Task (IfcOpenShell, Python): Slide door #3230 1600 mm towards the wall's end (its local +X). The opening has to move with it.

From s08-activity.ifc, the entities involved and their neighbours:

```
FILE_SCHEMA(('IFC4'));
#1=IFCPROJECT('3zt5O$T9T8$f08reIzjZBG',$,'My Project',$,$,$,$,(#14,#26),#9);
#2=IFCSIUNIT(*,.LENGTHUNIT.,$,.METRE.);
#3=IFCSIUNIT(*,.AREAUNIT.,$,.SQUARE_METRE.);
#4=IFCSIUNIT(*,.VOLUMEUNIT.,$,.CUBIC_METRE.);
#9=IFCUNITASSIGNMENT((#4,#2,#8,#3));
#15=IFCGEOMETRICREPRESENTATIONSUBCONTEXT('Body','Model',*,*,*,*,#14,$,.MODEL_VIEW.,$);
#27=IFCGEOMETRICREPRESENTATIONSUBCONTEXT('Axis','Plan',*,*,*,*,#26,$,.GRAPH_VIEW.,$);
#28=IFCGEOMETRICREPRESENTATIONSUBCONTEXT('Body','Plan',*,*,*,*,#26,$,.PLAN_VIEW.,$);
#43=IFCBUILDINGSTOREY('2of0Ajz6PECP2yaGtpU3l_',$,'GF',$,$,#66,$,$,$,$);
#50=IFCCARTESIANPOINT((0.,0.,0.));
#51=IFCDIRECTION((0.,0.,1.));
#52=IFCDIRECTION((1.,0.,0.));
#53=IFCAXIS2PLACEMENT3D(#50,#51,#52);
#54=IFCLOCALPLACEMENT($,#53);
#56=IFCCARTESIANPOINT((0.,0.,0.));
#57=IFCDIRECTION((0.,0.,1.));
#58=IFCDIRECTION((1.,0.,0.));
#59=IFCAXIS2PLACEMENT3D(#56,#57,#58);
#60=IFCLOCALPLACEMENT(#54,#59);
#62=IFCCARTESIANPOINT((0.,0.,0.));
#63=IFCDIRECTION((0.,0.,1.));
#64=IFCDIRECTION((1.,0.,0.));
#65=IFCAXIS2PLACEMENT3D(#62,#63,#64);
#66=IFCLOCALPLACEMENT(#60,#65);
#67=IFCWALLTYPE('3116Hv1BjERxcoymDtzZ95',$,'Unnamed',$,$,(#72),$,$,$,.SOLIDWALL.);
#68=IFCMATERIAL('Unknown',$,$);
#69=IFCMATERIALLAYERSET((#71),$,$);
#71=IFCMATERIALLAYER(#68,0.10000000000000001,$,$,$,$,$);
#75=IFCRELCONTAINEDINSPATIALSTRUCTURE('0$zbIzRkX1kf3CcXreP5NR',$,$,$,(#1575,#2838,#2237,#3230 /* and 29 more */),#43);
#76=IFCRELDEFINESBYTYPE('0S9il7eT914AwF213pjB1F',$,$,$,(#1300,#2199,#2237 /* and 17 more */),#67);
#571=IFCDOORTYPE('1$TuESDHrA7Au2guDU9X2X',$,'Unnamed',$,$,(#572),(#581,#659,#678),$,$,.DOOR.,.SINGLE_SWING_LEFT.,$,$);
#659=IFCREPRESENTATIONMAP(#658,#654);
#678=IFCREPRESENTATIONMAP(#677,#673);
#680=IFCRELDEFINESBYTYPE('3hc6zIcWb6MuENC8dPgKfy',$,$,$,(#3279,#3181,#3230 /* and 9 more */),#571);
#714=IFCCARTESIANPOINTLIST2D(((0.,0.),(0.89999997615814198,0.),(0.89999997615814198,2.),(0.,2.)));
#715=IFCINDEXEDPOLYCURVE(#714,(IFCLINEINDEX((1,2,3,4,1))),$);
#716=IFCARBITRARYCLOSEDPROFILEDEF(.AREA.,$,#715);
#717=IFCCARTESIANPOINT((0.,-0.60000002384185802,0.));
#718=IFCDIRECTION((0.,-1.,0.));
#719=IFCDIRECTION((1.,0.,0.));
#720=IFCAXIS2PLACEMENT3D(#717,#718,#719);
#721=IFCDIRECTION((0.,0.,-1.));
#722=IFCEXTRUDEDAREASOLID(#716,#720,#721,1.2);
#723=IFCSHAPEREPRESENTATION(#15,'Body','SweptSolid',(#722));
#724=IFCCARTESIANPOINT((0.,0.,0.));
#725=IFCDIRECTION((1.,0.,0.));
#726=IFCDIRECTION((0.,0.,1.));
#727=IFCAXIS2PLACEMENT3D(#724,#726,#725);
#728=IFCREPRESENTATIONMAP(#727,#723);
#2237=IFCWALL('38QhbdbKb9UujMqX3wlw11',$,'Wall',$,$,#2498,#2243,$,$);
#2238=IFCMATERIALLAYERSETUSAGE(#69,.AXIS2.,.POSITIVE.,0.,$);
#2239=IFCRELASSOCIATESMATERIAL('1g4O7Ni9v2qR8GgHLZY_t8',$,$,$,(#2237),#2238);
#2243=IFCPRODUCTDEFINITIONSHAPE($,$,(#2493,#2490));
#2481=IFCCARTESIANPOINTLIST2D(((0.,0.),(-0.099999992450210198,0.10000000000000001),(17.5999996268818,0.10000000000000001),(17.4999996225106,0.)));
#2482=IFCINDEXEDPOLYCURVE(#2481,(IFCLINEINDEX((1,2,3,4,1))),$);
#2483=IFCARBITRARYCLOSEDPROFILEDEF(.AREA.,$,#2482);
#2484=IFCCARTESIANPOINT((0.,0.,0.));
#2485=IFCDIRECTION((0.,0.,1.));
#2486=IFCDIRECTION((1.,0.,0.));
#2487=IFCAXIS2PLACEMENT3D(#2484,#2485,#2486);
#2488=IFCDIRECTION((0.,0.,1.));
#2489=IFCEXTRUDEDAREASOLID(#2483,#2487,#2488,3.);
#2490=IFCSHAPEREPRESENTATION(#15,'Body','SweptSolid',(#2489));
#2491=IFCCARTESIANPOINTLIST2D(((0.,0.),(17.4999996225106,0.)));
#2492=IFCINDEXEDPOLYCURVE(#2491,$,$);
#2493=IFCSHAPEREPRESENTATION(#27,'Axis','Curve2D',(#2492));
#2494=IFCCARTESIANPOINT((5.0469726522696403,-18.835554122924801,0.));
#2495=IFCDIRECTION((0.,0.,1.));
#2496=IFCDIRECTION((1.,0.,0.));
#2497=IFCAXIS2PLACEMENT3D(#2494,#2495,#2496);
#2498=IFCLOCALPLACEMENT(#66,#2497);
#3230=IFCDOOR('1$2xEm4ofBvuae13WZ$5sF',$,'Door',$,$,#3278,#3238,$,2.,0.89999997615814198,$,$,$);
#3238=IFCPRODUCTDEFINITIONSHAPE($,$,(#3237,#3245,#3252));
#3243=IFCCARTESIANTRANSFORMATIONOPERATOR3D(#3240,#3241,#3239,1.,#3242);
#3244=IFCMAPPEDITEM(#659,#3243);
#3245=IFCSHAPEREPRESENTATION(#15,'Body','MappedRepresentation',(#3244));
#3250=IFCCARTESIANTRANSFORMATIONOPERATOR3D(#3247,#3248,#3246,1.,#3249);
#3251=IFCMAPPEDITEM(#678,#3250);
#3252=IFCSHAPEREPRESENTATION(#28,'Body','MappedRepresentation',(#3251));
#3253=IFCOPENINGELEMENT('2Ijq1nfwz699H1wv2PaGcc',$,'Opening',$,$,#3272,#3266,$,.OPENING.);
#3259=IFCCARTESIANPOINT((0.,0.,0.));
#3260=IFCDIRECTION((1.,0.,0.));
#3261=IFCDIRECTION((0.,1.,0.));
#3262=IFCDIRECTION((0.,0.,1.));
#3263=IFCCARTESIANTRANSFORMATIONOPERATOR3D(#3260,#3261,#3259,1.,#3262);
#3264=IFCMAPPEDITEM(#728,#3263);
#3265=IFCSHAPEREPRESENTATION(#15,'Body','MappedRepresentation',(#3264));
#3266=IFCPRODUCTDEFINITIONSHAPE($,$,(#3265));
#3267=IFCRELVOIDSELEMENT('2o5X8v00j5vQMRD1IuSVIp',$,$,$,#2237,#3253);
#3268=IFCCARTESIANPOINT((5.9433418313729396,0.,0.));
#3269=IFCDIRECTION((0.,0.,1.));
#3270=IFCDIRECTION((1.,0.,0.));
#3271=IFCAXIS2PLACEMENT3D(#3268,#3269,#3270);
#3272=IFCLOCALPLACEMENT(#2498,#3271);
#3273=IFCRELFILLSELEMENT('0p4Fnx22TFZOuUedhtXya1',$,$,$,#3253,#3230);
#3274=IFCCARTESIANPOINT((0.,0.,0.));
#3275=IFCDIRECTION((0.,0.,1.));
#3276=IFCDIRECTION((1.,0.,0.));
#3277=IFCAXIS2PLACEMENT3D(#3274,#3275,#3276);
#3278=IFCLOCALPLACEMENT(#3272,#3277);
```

```python
import ifcopenshell
import ifcopenshell.api.geometry
import ifcopenshell.util.placement

model = ifcopenshell.open("s08-activity.ifc")

door = model.by_id(3230)
opening = door.FillsVoids[0].RelatingOpeningElement
wall = opening.VoidsElements[0].RelatingBuildingElement

wall_matrix = ifcopenshell.util.placement.get_local_placement(wall.ObjectPlacement)
shift = wall_matrix[:3, 0] * 1.6
before = ifcopenshell.util.placement.get_local_placement(door.ObjectPlacement)[:3, 3].copy()

# The door is placed relative to its opening, so it follows when the opening moves.
matrix = ifcopenshell.util.placement.get_local_placement(opening.ObjectPlacement)
matrix[:3, 3] += shift
ifcopenshell.api.geometry.edit_object_placement(
    model, product=opening, matrix=matrix, is_si=False, should_transform_children=True
)

after = ifcopenshell.util.placement.get_local_placement(door.ObjectPlacement)[:3, 3]
print("door moved by", (after - before).round(3) + 0.0)

model.write("s08-activity-out.ifc")
```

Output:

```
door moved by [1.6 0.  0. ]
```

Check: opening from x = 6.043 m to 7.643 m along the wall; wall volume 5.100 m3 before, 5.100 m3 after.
